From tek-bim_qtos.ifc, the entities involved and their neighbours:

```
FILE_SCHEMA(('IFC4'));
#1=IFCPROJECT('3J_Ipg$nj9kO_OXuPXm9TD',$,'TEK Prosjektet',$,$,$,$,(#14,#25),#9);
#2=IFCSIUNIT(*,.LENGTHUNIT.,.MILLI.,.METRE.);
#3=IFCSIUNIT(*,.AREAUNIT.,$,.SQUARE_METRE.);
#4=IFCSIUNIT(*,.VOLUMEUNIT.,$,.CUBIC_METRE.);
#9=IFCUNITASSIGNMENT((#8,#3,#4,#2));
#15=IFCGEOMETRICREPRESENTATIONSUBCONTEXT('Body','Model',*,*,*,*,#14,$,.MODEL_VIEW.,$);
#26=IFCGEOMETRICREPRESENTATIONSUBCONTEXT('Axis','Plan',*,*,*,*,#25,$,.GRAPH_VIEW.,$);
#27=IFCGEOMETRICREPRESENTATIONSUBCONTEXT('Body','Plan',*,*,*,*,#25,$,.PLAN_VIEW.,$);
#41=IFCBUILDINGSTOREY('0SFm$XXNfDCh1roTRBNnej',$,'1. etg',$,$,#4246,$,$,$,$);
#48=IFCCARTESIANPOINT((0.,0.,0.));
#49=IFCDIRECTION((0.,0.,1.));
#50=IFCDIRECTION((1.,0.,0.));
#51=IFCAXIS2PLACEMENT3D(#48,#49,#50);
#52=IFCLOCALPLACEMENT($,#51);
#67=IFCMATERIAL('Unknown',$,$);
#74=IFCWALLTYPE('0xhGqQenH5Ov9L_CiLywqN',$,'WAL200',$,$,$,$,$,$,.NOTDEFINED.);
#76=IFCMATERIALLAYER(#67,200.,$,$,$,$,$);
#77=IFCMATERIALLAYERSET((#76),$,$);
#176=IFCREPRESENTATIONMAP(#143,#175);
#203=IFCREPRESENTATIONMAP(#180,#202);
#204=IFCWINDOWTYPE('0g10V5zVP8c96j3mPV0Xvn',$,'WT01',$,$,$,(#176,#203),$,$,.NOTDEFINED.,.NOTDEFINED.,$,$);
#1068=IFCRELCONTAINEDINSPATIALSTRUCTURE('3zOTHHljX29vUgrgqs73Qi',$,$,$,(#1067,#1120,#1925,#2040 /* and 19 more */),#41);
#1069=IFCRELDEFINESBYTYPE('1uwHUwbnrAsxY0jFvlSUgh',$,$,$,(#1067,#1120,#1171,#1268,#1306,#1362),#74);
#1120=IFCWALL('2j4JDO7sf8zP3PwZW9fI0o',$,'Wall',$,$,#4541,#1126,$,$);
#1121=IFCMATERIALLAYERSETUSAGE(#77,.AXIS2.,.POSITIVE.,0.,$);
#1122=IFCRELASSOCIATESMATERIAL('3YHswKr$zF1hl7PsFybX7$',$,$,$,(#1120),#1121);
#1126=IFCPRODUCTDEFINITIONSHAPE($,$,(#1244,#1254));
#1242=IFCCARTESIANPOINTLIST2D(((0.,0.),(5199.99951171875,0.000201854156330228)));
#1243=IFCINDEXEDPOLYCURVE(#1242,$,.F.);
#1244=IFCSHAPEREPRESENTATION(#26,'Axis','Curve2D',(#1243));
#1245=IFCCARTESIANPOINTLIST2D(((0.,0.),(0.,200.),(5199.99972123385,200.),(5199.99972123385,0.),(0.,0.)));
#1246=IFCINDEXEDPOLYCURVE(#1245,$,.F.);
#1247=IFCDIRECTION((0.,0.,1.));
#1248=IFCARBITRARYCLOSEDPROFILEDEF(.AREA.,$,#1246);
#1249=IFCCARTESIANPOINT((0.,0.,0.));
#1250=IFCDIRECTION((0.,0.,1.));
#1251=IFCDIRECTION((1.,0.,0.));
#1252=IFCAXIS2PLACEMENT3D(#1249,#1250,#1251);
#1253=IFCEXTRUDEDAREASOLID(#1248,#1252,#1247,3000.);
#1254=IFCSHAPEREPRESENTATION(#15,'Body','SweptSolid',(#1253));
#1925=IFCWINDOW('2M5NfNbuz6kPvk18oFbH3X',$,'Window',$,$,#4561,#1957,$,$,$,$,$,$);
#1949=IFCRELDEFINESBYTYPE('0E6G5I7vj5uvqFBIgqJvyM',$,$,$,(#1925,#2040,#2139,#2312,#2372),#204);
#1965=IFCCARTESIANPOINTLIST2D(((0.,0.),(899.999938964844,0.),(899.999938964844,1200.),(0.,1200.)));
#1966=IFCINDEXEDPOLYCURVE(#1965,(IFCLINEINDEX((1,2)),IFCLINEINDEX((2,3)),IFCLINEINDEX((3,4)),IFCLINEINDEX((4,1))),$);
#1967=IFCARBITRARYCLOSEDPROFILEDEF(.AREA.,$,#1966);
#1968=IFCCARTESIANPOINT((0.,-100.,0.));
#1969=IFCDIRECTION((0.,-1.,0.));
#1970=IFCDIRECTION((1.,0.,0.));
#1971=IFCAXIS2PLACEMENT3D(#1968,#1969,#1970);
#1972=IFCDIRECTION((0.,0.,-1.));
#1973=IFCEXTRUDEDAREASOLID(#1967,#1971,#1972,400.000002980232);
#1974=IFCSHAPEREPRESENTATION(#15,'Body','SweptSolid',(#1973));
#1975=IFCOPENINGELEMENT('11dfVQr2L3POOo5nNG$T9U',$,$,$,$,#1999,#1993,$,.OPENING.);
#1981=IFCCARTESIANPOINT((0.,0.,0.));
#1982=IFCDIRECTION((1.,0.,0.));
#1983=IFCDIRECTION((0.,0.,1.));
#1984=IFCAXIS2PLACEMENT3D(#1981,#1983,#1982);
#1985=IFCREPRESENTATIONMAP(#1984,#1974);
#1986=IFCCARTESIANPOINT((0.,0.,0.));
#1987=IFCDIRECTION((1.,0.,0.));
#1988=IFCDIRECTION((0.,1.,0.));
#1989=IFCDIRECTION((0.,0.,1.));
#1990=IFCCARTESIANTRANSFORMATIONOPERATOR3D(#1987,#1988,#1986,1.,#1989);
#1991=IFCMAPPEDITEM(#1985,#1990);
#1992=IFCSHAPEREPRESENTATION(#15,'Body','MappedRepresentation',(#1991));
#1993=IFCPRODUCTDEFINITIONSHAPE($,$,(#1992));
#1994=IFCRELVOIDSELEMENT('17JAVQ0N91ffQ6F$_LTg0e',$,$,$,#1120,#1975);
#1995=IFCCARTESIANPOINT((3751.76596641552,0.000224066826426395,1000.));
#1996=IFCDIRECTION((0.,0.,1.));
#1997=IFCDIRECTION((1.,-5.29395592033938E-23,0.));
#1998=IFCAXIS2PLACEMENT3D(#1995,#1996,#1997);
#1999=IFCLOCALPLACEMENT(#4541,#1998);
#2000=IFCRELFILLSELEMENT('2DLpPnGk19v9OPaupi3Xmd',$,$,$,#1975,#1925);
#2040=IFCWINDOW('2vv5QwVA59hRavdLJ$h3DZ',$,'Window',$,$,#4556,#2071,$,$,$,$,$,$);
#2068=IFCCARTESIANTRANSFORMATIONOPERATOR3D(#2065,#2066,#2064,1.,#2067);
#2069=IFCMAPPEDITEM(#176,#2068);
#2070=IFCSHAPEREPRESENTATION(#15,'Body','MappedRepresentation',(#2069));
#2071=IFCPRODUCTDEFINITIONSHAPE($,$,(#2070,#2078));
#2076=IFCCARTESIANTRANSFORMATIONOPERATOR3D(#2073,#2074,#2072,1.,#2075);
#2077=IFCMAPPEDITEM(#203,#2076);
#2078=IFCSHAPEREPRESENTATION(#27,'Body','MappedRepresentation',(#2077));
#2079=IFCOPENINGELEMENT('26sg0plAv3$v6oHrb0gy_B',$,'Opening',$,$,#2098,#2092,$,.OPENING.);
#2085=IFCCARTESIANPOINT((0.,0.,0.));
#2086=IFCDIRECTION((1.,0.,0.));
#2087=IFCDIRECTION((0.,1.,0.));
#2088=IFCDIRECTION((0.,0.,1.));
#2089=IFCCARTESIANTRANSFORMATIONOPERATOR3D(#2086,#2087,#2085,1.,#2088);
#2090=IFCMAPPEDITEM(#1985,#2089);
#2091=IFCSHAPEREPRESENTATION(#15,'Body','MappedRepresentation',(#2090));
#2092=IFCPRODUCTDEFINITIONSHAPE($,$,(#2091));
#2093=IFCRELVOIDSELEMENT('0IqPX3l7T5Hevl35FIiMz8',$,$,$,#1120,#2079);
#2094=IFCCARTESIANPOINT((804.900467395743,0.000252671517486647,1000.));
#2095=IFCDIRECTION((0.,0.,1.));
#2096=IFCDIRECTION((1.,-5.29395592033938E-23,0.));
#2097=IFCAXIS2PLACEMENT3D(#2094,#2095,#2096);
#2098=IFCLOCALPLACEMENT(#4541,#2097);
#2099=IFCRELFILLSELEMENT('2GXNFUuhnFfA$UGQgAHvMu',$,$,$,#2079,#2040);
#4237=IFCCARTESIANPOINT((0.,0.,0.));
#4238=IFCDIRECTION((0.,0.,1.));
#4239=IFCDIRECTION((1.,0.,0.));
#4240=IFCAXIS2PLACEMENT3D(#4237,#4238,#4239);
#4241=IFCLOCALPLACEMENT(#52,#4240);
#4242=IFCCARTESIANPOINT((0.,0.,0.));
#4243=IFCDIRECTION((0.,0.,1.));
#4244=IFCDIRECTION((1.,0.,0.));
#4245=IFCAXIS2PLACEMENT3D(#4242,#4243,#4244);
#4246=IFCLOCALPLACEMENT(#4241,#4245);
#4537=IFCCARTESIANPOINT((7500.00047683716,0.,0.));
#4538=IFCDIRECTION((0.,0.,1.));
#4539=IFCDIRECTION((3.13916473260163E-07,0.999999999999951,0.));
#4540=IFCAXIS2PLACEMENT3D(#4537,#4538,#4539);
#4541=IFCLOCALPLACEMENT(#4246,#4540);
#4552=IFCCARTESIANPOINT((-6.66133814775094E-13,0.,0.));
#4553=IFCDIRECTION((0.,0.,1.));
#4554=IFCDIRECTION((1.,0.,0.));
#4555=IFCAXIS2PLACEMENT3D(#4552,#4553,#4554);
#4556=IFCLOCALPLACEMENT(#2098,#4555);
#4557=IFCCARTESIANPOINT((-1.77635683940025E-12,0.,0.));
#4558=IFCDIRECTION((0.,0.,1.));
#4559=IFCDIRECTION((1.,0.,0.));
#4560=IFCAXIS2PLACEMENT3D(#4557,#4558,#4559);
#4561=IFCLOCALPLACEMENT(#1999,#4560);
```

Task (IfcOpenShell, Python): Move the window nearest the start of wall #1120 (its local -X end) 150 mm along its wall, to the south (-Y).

```python
import ifcopenshell
import ifcopenshell.api.geometry
import ifcopenshell.util.placement

model = ifcopenshell.open("tek-bim_qtos.ifc")

window = model.by_guid("2vv5QwVA59hRavdLJ$h3DZ")
opening = window.FillsVoids[0].RelatingOpeningElement
wall = opening.VoidsElements[0].RelatingBuildingElement

wall_matrix = ifcopenshell.util.placement.get_local_placement(wall.ObjectPlacement)
shift = wall_matrix[:3, 0] * -150.0
before = ifcopenshell.util.placement.get_local_placement(window.ObjectPlacement)[:3, 3].copy()

# The window is placed relative to its opening, so it follows when the opening moves.
matrix = ifcopenshell.util.placement.get_local_placement(opening.ObjectPlacement)
matrix[:3, 3] += shift
ifcopenshell.api.geometry.edit_object_placement(
    model, product=opening, matrix=matrix, is_si=False, should_transform_children=True
)

after = ifcopenshell.util.placement.get_local_placement(window.ObjectPlacement)[:3, 3]
print("window moved by", (after - before).round(3) + 0.0)

model.write("tek-bim_qtos_rev.ifc")
```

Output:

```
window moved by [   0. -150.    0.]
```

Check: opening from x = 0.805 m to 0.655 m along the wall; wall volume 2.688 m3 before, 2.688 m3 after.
